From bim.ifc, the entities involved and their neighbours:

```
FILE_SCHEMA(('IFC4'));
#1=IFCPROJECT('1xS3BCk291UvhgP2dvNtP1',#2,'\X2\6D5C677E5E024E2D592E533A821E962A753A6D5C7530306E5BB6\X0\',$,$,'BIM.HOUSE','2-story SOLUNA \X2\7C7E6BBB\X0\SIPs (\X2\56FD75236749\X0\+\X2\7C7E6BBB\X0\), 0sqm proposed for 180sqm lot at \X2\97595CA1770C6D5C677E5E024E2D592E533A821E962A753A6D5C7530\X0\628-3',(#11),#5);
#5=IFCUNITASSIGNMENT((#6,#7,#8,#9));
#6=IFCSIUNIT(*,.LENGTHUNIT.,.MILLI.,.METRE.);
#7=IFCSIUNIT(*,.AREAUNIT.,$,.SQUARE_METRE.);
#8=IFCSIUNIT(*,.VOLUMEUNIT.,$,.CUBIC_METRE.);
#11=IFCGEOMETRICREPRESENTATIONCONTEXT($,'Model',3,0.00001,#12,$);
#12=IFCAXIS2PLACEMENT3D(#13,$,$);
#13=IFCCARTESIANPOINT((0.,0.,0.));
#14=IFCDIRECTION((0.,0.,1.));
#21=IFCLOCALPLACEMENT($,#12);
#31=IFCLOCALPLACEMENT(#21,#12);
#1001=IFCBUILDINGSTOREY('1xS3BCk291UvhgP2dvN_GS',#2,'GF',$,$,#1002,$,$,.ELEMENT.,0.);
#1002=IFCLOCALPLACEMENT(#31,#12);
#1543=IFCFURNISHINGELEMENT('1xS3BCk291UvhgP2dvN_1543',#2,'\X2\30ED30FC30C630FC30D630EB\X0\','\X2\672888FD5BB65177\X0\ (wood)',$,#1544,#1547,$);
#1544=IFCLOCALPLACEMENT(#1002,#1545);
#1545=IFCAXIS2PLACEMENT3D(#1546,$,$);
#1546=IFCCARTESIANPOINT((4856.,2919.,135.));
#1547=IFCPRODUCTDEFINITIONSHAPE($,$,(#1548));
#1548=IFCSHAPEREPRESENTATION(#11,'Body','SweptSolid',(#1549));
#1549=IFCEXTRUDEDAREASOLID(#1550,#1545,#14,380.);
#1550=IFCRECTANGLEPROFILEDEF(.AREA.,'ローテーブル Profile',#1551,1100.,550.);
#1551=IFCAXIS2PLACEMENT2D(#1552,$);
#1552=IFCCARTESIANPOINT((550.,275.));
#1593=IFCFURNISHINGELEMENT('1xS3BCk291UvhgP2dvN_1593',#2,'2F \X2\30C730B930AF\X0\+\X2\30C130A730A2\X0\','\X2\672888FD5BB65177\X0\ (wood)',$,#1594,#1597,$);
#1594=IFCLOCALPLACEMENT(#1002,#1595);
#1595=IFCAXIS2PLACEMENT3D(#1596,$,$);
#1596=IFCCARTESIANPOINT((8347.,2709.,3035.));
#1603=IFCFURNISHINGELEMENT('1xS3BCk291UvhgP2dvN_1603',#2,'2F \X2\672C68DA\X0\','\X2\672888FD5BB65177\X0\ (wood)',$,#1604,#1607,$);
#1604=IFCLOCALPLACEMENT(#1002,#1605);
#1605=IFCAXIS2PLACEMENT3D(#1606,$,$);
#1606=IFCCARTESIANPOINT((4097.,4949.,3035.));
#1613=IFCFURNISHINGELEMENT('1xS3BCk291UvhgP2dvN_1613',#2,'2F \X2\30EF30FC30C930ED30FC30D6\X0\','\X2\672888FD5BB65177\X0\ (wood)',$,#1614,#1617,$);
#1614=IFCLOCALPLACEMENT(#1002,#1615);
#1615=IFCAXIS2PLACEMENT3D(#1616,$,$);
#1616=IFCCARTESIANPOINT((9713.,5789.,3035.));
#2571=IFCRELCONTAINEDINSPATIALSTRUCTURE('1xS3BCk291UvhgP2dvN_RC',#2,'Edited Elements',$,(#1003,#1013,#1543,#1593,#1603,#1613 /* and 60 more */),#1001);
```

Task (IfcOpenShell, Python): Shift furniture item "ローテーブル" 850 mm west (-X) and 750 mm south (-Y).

```python
import ifcopenshell
import ifcopenshell.api.geometry
import ifcopenshell.util.placement
import ifcopenshell.util.unit

model = ifcopenshell.open("bim.ifc")
unit_scale = ifcopenshell.util.unit.calculate_unit_scale(model)

item = model.by_guid("1xS3BCk291UvhgP2dvN_1543")
matrix = ifcopenshell.util.placement.get_local_placement(item.ObjectPlacement)
matrix[0, 3] -= 0.85 / unit_scale
matrix[1, 3] -= 0.75 / unit_scale
ifcopenshell.api.geometry.edit_object_placement(model, product=item, matrix=matrix, is_si=False)

print(ifcopenshell.util.placement.get_local_placement(item.ObjectPlacement).round(3) + 0.0)

model.write("bim-out.ifc")
```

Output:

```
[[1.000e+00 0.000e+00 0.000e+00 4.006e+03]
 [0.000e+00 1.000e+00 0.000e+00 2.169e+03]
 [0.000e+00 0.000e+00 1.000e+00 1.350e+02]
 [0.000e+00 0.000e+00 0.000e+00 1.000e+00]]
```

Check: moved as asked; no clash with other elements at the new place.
